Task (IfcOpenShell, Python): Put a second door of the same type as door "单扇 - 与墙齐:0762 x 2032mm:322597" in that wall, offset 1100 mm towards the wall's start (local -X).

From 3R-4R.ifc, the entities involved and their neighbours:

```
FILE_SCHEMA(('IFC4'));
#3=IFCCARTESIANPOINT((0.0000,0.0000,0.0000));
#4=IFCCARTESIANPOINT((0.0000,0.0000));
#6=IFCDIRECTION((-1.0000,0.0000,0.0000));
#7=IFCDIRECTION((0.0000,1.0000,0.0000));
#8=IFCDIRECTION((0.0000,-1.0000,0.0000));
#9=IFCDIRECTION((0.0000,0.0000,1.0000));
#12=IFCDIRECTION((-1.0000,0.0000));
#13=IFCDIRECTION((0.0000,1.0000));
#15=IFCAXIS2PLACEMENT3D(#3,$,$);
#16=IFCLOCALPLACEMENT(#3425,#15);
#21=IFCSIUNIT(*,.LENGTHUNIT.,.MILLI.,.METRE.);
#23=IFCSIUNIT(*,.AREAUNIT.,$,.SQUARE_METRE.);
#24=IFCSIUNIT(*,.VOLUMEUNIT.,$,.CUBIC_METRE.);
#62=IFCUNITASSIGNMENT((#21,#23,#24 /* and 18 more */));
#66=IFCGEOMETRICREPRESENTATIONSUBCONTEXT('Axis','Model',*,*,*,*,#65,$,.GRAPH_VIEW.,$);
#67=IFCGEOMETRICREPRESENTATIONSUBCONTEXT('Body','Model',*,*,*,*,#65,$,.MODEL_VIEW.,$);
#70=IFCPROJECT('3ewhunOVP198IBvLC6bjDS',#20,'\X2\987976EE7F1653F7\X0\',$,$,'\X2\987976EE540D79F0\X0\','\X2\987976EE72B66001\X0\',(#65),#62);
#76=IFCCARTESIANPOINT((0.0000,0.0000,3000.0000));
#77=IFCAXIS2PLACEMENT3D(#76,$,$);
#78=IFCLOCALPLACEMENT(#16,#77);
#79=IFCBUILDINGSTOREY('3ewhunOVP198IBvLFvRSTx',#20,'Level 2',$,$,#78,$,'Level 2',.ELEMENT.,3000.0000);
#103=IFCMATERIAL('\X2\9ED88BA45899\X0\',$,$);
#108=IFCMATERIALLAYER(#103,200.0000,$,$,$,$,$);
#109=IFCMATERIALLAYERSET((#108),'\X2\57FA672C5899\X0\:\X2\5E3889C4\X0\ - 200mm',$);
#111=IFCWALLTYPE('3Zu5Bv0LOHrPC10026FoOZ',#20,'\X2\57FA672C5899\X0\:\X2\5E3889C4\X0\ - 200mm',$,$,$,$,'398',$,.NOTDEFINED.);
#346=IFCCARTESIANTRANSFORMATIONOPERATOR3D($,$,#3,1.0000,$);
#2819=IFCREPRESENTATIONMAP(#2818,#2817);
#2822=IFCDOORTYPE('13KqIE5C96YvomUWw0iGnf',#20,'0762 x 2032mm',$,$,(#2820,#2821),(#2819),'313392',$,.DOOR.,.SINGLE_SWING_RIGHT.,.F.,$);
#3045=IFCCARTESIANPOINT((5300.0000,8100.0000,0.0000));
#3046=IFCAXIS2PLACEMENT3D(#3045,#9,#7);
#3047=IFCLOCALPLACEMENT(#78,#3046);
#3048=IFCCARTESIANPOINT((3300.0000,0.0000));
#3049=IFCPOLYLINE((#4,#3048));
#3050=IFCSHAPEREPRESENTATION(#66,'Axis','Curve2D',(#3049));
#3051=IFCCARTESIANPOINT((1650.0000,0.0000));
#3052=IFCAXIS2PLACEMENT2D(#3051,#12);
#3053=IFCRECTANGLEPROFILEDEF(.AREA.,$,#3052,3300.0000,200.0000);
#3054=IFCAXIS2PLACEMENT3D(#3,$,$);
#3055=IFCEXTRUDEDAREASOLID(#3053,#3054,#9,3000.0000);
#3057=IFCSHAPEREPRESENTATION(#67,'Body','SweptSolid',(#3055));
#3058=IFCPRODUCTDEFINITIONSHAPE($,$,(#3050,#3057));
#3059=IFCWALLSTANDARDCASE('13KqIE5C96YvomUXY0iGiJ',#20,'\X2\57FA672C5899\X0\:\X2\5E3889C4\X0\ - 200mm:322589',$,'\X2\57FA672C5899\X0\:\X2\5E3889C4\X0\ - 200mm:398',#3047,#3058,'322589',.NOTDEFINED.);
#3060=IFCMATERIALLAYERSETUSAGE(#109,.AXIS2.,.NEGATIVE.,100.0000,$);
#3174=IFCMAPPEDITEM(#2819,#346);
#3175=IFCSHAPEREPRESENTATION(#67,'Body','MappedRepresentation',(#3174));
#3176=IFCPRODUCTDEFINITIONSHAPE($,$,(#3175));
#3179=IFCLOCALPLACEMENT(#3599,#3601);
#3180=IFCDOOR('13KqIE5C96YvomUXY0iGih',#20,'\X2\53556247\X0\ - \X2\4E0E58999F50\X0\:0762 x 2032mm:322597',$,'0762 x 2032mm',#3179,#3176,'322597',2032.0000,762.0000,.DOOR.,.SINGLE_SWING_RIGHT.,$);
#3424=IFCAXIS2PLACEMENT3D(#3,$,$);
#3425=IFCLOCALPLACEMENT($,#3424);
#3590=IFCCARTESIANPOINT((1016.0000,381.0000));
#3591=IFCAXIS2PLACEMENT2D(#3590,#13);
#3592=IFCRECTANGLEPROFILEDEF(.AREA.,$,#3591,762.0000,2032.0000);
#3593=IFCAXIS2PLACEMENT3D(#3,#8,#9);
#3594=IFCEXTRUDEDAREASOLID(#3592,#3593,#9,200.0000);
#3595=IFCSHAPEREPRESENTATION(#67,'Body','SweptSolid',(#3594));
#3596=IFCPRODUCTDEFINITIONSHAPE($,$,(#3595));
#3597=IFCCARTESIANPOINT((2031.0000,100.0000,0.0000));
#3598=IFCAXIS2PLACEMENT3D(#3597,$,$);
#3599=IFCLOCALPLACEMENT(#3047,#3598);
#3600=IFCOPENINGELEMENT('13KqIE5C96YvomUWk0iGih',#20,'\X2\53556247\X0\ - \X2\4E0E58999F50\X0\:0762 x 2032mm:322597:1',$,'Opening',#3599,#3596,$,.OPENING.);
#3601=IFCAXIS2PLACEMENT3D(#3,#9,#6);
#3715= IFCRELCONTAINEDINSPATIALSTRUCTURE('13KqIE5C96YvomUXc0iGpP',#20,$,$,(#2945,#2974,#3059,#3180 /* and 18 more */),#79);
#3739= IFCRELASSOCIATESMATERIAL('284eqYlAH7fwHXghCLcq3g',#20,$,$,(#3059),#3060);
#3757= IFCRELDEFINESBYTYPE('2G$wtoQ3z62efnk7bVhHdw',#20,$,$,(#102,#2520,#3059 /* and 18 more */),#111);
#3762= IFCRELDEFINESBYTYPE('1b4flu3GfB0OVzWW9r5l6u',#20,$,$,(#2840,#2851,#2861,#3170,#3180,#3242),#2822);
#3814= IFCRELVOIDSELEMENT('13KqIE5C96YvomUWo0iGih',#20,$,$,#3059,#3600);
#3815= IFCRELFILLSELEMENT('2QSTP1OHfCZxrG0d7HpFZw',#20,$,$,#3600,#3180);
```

```python
import ifcopenshell
import ifcopenshell.api.feature
import ifcopenshell.api.geometry
import ifcopenshell.api.root
import ifcopenshell.geom
import ifcopenshell.util.element
import ifcopenshell.util.placement
import ifcopenshell.util.shape
import ifcopenshell.util.unit

model = ifcopenshell.open("3R-4R.ifc")
unit_scale = ifcopenshell.util.unit.calculate_unit_scale(model)
settings = ifcopenshell.geom.settings()


def volume(element):
    """Net volume in cubic metres, openings subtracted."""
    shape = ifcopenshell.geom.create_shape(settings, element)
    return ifcopenshell.util.shape.get_volume(shape.geometry)


def reuse_history(source, copy):
    """copy_class also copies each property set's owner history, people and application; keep the originals."""
    for rel in copy.IsDefinedBy:
        if rel.is_a("IfcRelDefinesByProperties") and (history := rel.RelatingPropertyDefinition.OwnerHistory):
            rel.RelatingPropertyDefinition.OwnerHistory = source.OwnerHistory
            ifcopenshell.util.element.remove_deep2(model, history)


door = model.by_guid("13KqIE5C96YvomUXY0iGih")
opening = door.FillsVoids[0].RelatingOpeningElement
wall = opening.VoidsElements[0].RelatingBuildingElement
before = volume(wall)
shift = ifcopenshell.util.placement.get_local_placement(wall.ObjectPlacement)[:3, 0] * -1.1 / unit_scale

# copy_class copies the void relationship, type, container and properties, but no geometry.
new_opening = ifcopenshell.api.root.copy_class(model, product=opening)
new_opening.Representation = ifcopenshell.util.element.copy_deep(
    model, opening.Representation, exclude=["IfcGeometricRepresentationContext", "IfcRepresentationMap"]
)
new_opening.Name = "单扇 - 与墙齐:0762 x 2032mm"
new_door = ifcopenshell.api.root.copy_class(model, product=door)
new_door.Representation = ifcopenshell.util.element.copy_deep(
    model, door.Representation, exclude=["IfcGeometricRepresentationContext", "IfcRepresentationMap"]
)
new_door.Name = "单扇 - 与墙齐:0762 x 2032mm"
new_door.Tag = None
reuse_history(door, new_door)
ifcopenshell.api.feature.add_filling(model, opening=new_opening, element=new_door)

for old, new in ((opening, new_opening), (door, new_door)):
    matrix = ifcopenshell.util.placement.get_local_placement(old.ObjectPlacement)
    matrix[:3, 3] += shift
    ifcopenshell.api.geometry.edit_object_placement(model, product=new, matrix=matrix, is_si=False)

after = volume(wall)

print(f"wall volume {before:.3f} -> {after:.3f} m3")

model.write("3R-4R_updated.ifc")
```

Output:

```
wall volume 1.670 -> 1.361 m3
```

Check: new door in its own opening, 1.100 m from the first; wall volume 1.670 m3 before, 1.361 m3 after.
